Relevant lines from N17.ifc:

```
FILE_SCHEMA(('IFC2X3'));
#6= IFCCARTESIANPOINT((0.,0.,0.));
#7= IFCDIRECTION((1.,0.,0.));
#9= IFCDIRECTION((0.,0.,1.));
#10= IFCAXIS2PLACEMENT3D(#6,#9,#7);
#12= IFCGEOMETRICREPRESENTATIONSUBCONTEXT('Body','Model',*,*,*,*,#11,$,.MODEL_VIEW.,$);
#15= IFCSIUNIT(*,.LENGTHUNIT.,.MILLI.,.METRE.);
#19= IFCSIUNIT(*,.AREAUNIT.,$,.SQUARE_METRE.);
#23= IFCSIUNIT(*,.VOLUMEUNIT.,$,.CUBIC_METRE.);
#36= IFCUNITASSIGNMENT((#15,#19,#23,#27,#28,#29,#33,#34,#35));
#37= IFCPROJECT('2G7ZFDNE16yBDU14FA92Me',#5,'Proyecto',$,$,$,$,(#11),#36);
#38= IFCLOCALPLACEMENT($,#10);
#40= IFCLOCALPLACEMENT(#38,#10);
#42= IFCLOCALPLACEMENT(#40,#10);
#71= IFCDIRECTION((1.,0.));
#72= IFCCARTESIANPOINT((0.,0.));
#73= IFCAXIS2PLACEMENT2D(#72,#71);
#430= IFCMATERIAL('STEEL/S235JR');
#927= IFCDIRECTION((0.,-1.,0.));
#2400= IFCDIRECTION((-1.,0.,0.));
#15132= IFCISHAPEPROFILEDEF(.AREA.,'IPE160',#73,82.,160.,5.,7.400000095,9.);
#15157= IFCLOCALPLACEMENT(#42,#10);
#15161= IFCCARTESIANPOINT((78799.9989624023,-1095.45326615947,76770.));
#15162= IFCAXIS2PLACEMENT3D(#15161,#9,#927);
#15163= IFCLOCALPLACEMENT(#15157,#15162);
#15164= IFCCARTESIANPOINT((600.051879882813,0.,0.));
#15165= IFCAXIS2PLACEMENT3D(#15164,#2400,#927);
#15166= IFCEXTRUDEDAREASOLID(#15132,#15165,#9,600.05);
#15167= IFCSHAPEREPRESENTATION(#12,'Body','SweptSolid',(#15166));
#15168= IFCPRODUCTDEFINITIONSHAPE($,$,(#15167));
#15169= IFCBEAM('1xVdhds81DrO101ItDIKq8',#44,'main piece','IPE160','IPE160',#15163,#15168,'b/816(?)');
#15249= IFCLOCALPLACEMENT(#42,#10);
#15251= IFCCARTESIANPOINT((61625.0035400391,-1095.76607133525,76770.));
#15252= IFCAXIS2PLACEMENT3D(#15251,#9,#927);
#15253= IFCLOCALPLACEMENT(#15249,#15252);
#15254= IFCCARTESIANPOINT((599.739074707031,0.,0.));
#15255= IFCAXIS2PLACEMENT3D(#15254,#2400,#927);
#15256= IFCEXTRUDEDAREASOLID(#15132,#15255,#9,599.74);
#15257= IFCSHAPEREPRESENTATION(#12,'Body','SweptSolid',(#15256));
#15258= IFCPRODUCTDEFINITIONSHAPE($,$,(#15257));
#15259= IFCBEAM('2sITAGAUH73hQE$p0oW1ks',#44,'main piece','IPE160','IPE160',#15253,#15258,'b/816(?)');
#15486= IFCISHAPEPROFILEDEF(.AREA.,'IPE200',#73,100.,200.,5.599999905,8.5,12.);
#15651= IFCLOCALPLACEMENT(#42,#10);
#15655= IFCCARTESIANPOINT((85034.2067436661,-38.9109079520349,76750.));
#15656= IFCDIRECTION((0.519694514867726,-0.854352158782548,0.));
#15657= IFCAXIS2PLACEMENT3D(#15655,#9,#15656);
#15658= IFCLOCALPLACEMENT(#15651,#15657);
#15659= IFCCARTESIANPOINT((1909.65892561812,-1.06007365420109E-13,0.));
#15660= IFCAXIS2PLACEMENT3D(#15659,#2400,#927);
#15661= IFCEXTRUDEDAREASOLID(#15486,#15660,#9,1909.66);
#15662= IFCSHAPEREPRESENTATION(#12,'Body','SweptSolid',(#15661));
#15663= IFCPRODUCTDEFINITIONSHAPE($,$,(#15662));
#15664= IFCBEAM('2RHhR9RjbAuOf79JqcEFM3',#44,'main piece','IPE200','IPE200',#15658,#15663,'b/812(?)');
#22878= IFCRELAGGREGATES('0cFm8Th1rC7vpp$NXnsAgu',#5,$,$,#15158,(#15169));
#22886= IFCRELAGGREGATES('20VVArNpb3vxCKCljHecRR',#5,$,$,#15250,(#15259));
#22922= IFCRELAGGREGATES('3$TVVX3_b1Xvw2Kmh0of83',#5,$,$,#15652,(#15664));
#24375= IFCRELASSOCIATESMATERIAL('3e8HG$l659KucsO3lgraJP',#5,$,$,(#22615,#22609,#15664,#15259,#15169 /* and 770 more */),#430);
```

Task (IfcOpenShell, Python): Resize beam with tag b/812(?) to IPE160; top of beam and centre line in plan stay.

```python
import ifcopenshell
import ifcopenshell.util.element
import ifcopenshell.util.representation

model = ifcopenshell.open("N17.ifc")

member = model.by_guid("2RHhR9RjbAuOf79JqcEFM3")
source = next(p for p in model.by_type("IfcIShapeProfileDef") if p.ProfileName == "IPE160")

body = ifcopenshell.util.representation.get_representation(member, "Model", "Body")
solid = body.Items[0]
old_profile = solid.SweptArea

# Copy the section's sizes but keep this member's own profile position.
profile = ifcopenshell.util.element.copy(model, source)
# Profiles are centred, so shift by half the change in depth to hold the top.
shift = (old_profile.OverallDepth - profile.OverallDepth) / 2
x, y = old_profile.Position.Location.Coordinates
up = (0.0, 1.0)  # upwards, in the solid's own plane
location = model.createIfcCartesianPoint((x + up[0] * shift, y + up[1] * shift))
profile.Position = model.createIfcAxis2Placement2D(location, old_profile.Position.RefDirection)
solid.SweptArea = profile
if not model.get_total_inverses(old_profile):
    ifcopenshell.util.element.remove_deep2(model, old_profile)
member.Description = member.Description.replace("IPE200", "IPE160")
member.ObjectType = member.ObjectType.replace("IPE200", "IPE160")

print(solid.SweptArea)

model.write("N17_updated.ifc")
```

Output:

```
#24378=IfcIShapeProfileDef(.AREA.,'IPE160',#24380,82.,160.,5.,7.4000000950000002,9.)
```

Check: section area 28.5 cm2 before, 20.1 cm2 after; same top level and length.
